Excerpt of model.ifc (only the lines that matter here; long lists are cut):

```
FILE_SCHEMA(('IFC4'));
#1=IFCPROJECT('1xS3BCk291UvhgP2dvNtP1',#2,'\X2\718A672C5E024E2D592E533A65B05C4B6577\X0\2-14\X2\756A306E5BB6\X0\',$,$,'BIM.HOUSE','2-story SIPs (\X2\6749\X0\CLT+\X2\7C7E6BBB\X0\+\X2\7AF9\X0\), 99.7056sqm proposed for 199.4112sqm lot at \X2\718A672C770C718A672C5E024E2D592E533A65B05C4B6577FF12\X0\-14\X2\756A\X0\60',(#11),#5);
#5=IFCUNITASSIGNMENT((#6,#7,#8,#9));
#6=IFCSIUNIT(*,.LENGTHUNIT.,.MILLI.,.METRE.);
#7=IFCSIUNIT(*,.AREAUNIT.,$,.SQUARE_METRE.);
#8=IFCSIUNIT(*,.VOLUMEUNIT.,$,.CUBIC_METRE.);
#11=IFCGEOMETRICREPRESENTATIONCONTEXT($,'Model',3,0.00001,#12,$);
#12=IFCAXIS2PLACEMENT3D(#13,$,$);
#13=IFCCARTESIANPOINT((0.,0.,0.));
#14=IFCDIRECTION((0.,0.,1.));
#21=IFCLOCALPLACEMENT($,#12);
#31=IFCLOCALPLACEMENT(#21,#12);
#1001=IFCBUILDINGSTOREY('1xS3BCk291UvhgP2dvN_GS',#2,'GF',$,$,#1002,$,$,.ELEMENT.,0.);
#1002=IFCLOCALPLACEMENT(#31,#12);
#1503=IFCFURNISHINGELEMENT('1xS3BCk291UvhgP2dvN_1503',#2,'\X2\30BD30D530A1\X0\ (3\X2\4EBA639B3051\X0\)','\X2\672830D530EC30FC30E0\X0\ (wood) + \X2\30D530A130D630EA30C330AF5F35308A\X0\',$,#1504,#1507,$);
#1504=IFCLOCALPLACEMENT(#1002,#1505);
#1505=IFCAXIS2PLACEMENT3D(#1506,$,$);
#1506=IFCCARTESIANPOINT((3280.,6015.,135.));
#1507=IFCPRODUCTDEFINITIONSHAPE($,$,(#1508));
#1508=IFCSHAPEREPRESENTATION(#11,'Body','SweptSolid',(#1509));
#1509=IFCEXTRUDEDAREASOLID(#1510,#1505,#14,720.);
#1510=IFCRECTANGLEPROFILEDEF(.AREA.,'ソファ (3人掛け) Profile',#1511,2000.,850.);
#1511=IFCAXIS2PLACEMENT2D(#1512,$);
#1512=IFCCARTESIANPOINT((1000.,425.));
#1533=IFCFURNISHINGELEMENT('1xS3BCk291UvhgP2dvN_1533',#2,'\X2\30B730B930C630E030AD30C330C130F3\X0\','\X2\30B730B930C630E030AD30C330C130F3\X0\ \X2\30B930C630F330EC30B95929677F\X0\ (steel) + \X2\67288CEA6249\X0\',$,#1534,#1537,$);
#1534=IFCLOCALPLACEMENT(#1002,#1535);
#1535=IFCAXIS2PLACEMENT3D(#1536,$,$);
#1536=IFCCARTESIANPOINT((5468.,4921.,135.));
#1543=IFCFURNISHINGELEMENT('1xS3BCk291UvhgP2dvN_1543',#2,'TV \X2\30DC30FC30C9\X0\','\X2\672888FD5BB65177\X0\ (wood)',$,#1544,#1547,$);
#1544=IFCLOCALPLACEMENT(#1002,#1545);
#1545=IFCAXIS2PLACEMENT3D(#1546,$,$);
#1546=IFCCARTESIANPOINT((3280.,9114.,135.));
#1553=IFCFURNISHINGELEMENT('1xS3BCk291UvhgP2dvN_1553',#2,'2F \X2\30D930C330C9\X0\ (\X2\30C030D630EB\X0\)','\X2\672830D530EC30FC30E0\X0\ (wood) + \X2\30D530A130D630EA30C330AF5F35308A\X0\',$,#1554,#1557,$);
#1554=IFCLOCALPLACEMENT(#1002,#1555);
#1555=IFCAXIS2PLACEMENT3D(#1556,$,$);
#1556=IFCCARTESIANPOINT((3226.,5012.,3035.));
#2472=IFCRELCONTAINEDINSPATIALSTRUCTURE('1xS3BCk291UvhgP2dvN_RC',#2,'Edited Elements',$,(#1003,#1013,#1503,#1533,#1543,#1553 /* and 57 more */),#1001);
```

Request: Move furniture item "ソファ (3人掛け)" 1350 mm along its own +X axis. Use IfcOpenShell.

```python
import ifcopenshell
import ifcopenshell.api.geometry
import ifcopenshell.util.placement
import ifcopenshell.util.unit

model = ifcopenshell.open("model.ifc")
unit_scale = ifcopenshell.util.unit.calculate_unit_scale(model)

item = model.by_guid("1xS3BCk291UvhgP2dvN_1503")
matrix = ifcopenshell.util.placement.get_local_placement(item.ObjectPlacement)
matrix[:3, 3] += matrix[:3, 0] * 1.35 / unit_scale
ifcopenshell.api.geometry.edit_object_placement(model, product=item, matrix=matrix, is_si=False)

print(ifcopenshell.util.placement.get_local_placement(item.ObjectPlacement).round(3) + 0.0)

model.write("model_updated.ifc")
```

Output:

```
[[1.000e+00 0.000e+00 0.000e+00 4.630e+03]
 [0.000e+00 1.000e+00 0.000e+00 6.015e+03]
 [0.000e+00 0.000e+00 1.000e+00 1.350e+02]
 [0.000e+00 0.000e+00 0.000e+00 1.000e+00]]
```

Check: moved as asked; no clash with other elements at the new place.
